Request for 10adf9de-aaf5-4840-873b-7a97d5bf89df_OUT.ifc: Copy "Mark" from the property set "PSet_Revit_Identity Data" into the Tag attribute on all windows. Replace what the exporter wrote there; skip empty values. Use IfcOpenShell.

First a look at what the model holds.

```python
import ifcopenshell
import ifcopenshell.util.element

model = ifcopenshell.open("10adf9de-aaf5-4840-873b-7a97d5bf89df_OUT.ifc")
print(model.schema)
windows = model.by_type("IfcWindow")
print(len(windows), "windows")
for e in windows[:8]:
    source = ifcopenshell.util.element.get_pset(e, "PSet_Revit_Identity Data", "Mark")
    target = e.Tag
    print(e.id(), repr(source), repr(target), sep=" | ")
```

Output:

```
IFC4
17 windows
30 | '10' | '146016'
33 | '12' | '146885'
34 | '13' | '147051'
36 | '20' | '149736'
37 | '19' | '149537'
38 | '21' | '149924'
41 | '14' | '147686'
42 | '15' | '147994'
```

```python
import ifcopenshell
import ifcopenshell.util.element

model = ifcopenshell.open("10adf9de-aaf5-4840-873b-7a97d5bf89df_OUT.ifc")

count = 0
for e in model.by_type("IfcWindow"):
    value = ifcopenshell.util.element.get_pset(e, "PSet_Revit_Identity Data", "Mark")
    current = e.Tag
    if not value or not value.strip() or current == value:
        continue
    e.Tag = value
    count += 1

print(count, "windows updated")

model.write("10adf9de-aaf5-4840-873b-7a97d5bf89df_OUT-out.ifc")
```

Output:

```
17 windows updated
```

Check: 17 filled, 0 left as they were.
